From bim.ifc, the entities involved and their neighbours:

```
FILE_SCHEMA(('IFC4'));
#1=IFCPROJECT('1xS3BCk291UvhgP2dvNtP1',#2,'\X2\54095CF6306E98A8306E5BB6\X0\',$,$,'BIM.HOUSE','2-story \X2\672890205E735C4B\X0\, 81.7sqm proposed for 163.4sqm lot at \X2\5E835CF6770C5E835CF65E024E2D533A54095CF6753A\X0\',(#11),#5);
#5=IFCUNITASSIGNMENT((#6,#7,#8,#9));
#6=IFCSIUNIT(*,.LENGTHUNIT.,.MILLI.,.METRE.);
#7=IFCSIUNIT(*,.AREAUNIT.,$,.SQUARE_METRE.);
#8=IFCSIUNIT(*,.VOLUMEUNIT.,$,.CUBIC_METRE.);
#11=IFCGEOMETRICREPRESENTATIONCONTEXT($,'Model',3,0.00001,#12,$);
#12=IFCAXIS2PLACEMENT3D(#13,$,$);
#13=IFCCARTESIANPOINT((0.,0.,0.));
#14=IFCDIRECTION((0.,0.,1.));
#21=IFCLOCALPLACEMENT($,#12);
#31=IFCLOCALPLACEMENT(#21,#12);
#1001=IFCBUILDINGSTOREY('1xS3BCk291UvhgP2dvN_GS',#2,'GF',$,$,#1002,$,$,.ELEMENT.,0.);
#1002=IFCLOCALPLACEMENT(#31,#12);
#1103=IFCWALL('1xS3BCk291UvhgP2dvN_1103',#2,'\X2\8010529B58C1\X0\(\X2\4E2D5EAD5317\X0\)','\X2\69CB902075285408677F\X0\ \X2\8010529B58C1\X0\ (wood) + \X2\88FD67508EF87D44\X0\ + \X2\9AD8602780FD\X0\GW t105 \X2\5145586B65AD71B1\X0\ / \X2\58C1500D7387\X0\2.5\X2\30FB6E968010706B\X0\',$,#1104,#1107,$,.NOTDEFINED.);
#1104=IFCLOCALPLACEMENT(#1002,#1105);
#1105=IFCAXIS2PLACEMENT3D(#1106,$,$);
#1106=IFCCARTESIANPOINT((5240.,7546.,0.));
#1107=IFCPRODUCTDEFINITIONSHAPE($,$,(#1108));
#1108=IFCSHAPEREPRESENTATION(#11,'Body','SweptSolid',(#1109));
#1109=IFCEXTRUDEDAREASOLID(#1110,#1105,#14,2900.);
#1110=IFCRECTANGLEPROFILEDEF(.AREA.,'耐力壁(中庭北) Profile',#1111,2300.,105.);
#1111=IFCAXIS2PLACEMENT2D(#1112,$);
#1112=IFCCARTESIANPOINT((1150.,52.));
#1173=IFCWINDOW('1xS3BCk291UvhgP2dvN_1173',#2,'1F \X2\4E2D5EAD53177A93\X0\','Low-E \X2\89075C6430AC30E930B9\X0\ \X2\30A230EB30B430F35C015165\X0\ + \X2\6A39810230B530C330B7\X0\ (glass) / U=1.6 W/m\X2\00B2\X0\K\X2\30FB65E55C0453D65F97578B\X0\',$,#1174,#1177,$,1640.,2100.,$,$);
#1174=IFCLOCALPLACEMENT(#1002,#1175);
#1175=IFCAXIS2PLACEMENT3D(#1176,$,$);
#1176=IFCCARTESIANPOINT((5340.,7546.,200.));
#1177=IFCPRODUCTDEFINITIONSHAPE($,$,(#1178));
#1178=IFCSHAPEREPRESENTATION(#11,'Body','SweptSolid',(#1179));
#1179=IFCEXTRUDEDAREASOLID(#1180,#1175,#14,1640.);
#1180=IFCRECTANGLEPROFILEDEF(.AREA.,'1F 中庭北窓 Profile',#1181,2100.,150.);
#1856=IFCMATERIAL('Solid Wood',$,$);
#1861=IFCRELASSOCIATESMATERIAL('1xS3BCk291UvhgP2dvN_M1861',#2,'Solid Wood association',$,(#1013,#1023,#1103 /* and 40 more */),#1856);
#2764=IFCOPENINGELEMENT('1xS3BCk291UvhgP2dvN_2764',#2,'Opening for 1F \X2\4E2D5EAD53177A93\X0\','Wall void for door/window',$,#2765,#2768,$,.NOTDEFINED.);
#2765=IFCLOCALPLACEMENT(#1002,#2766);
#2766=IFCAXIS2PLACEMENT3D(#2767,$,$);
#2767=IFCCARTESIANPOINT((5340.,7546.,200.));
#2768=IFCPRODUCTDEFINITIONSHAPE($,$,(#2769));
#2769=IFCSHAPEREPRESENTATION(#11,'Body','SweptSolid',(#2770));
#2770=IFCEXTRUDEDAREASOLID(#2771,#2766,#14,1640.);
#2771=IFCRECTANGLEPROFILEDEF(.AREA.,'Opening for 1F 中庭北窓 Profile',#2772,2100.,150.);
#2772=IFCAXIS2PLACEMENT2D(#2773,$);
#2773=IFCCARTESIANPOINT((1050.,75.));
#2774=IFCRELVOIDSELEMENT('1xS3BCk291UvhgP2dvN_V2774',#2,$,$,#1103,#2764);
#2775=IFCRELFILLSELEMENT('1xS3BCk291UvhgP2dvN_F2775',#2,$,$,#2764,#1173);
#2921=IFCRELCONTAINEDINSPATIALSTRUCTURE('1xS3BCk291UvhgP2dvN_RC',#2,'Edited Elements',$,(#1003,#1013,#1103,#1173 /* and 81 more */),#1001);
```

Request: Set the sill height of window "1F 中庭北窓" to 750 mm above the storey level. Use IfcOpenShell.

```python
import numpy as np
import ifcopenshell
import ifcopenshell.api.geometry
import ifcopenshell.geom
import ifcopenshell.util.element
import ifcopenshell.util.placement
import ifcopenshell.util.shape
import ifcopenshell.util.unit

model = ifcopenshell.open("bim.ifc")
unit_scale = ifcopenshell.util.unit.calculate_unit_scale(model)

window = model.by_guid("1xS3BCk291UvhgP2dvN_1173")
opening = window.FillsVoids[0].RelatingOpeningElement
storey = ifcopenshell.util.element.get_container(window, ifc_class="IfcBuildingStorey")
level = ifcopenshell.util.placement.get_local_placement(storey.ObjectPlacement)[2, 3]

# The opening's origin need not be at the sill, so measure its lowest point.
shape = ifcopenshell.geom.create_shape(ifcopenshell.geom.settings(), opening)
bottom = ifcopenshell.util.shape.get_shape_bottom_elevation(shape, shape.geometry) / unit_scale
dz = level + 0.75 / unit_scale - bottom

shift = np.array([0.0, 0.0, dz])
# The window is not placed relative to its opening, so move both.
for product in (opening, window):
    matrix = ifcopenshell.util.placement.get_local_placement(product.ObjectPlacement)
    matrix[:3, 3] += shift
    ifcopenshell.api.geometry.edit_object_placement(model, product=product, matrix=matrix, is_si=False)

print(f"moved by {dz * unit_scale:+.3f} m")

model.write("bim_updated.ifc")
```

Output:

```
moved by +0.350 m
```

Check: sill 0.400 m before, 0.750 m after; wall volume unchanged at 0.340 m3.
